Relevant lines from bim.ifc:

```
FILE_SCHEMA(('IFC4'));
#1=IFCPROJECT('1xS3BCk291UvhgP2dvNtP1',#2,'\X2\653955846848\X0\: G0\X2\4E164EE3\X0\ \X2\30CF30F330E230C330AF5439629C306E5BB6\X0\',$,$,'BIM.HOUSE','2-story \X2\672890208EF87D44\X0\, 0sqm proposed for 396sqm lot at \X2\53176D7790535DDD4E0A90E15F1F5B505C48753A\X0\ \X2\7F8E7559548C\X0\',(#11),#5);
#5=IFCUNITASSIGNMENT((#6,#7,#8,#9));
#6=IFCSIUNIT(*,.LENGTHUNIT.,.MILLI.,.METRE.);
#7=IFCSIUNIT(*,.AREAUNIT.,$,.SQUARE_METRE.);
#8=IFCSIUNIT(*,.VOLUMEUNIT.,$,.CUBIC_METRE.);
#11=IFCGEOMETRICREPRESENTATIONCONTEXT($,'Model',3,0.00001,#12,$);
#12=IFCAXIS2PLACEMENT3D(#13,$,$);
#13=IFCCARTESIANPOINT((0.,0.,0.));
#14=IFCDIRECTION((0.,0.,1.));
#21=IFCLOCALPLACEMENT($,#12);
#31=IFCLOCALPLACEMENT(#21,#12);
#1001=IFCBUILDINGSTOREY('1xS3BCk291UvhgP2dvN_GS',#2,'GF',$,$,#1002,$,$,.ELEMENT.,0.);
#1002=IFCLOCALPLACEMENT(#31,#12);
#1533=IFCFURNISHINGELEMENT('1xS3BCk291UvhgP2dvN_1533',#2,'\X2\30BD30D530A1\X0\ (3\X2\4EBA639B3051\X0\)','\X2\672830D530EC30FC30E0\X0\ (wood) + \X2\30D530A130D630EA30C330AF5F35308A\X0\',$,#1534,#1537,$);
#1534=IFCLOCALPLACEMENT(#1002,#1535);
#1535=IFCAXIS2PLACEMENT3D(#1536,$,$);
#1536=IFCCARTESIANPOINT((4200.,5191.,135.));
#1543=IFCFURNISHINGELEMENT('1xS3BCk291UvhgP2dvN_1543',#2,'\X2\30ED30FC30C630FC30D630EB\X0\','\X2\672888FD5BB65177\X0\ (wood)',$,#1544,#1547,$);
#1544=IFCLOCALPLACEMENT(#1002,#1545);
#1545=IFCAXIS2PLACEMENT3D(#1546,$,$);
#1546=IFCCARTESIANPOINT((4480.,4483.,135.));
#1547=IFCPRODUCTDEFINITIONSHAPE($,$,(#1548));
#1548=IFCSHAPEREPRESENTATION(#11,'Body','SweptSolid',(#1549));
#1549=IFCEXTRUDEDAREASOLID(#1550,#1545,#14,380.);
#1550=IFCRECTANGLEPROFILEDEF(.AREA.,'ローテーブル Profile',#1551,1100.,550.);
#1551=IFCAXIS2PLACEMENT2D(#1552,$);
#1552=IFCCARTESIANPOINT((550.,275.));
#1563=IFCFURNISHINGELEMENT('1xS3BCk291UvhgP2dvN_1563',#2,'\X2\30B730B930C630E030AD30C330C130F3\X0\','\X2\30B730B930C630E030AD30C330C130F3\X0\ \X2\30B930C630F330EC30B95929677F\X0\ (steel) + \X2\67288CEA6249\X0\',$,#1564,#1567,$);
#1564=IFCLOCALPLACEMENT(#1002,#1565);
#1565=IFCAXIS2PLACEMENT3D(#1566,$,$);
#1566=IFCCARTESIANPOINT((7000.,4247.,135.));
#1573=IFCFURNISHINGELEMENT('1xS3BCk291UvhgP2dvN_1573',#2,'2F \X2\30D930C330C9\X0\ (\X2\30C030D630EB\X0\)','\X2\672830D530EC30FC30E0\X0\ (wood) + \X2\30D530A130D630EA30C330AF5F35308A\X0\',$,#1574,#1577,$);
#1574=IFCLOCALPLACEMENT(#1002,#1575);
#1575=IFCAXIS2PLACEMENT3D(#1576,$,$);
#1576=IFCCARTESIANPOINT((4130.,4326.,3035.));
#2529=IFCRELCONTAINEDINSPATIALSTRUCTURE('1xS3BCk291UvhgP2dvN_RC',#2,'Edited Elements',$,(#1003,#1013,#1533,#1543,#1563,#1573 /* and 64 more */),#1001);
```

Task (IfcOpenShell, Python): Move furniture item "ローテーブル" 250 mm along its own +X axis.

```python
import ifcopenshell
import ifcopenshell.api.geometry
import ifcopenshell.util.placement

model = ifcopenshell.open("bim.ifc")

item = model.by_guid("1xS3BCk291UvhgP2dvN_1543")
matrix = ifcopenshell.util.placement.get_local_placement(item.ObjectPlacement)
matrix[:3, 3] += matrix[:3, 0] * 250.0
ifcopenshell.api.geometry.edit_object_placement(model, product=item, matrix=matrix, is_si=False)

print(ifcopenshell.util.placement.get_local_placement(item.ObjectPlacement).round(3) + 0.0)

model.write("bim_updated.ifc")
```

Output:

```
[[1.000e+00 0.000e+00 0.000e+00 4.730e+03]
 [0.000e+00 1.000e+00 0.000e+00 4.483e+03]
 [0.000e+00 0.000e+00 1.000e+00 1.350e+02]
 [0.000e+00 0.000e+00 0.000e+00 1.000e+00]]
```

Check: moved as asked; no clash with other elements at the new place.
